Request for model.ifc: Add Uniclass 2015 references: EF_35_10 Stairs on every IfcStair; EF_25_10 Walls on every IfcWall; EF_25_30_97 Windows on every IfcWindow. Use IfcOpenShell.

First a look at what the model holds.

```python
import ifcopenshell

model = ifcopenshell.open("model.ifc")
print(model.schema)
print("classifications:", [c.Name for c in model.by_type("IfcClassification")])
for ifc_class in ("IfcDoor", "IfcRoof", "IfcStair", "IfcWall", "IfcWindow"):
    print(ifc_class, len(model.by_type(ifc_class)))
```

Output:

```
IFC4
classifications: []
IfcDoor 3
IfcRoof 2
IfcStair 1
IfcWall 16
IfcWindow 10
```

```python
import ifcopenshell
import ifcopenshell.api.classification

model = ifcopenshell.open("model.ifc")

system = ifcopenshell.api.classification.add_classification(model, classification="Uniclass 2015")

codes = {
    "IfcStair": ("EF_35_10", "Stairs"),
    "IfcWall": ("EF_25_10", "Walls"),
    "IfcWindow": ("EF_25_30_97", "Windows"),
}
for ifc_class, (code, name) in codes.items():
    products = model.by_type(ifc_class)
    ifcopenshell.api.classification.add_reference(
        model, products=products, classification=system, identification=code, name=name
    )
    print(code, len(products))

model.write("model_updated.ifc")
```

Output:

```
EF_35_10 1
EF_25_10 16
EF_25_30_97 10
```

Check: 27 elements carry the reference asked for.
